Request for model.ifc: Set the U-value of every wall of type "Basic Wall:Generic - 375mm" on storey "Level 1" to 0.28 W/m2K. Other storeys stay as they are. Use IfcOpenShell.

First a look at what the model holds.

```python
import ifcopenshell
import ifcopenshell.util.element

model = ifcopenshell.open("model.ifc")
print(model.schema)
storey = next(s for s in model.by_type("IfcBuildingStorey") if s.Name == "Level 1")
walls = [e for e in ifcopenshell.util.element.get_decomposition(storey) if e.is_a("IfcWall")]
seen = {}
for e in walls:
    element_type = ifcopenshell.util.element.get_type(e)
    key = (element_type.Name if element_type != e and element_type else None, ifcopenshell.util.element.get_pset(e, "Pset_WallCommon", "ThermalTransmittance"))
    seen[key] = seen.get(key, 0) + 1
for (name, value), count in sorted(seen.items(), key=str):
    print(count, "x", name, "|", value)
```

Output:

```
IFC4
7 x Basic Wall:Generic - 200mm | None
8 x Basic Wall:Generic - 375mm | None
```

```python
import ifcopenshell
import ifcopenshell.api.pset
import ifcopenshell.util.element

model = ifcopenshell.open("model.ifc")

storey = next(s for s in model.by_type("IfcBuildingStorey") if s.Name == "Level 1")
walls = [e for e in ifcopenshell.util.element.get_decomposition(storey) if e.is_a("IfcWall")]

count = 0
for e in walls:
    element_type = ifcopenshell.util.element.get_type(e)
    if element_type in (None, e) or element_type.Name != "Basic Wall:Generic - 375mm":
        continue
    # add_pset returns the element's existing set when there is one.
    pset = ifcopenshell.api.pset.add_pset(model, product=e, name="Pset_WallCommon")
    ifcopenshell.api.pset.edit_pset(model, pset=pset, properties={"ThermalTransmittance": 0.28})
    count += 1

print(count, "walls updated")

model.write("model_v2.ifc")
```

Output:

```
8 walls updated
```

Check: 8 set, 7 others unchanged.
